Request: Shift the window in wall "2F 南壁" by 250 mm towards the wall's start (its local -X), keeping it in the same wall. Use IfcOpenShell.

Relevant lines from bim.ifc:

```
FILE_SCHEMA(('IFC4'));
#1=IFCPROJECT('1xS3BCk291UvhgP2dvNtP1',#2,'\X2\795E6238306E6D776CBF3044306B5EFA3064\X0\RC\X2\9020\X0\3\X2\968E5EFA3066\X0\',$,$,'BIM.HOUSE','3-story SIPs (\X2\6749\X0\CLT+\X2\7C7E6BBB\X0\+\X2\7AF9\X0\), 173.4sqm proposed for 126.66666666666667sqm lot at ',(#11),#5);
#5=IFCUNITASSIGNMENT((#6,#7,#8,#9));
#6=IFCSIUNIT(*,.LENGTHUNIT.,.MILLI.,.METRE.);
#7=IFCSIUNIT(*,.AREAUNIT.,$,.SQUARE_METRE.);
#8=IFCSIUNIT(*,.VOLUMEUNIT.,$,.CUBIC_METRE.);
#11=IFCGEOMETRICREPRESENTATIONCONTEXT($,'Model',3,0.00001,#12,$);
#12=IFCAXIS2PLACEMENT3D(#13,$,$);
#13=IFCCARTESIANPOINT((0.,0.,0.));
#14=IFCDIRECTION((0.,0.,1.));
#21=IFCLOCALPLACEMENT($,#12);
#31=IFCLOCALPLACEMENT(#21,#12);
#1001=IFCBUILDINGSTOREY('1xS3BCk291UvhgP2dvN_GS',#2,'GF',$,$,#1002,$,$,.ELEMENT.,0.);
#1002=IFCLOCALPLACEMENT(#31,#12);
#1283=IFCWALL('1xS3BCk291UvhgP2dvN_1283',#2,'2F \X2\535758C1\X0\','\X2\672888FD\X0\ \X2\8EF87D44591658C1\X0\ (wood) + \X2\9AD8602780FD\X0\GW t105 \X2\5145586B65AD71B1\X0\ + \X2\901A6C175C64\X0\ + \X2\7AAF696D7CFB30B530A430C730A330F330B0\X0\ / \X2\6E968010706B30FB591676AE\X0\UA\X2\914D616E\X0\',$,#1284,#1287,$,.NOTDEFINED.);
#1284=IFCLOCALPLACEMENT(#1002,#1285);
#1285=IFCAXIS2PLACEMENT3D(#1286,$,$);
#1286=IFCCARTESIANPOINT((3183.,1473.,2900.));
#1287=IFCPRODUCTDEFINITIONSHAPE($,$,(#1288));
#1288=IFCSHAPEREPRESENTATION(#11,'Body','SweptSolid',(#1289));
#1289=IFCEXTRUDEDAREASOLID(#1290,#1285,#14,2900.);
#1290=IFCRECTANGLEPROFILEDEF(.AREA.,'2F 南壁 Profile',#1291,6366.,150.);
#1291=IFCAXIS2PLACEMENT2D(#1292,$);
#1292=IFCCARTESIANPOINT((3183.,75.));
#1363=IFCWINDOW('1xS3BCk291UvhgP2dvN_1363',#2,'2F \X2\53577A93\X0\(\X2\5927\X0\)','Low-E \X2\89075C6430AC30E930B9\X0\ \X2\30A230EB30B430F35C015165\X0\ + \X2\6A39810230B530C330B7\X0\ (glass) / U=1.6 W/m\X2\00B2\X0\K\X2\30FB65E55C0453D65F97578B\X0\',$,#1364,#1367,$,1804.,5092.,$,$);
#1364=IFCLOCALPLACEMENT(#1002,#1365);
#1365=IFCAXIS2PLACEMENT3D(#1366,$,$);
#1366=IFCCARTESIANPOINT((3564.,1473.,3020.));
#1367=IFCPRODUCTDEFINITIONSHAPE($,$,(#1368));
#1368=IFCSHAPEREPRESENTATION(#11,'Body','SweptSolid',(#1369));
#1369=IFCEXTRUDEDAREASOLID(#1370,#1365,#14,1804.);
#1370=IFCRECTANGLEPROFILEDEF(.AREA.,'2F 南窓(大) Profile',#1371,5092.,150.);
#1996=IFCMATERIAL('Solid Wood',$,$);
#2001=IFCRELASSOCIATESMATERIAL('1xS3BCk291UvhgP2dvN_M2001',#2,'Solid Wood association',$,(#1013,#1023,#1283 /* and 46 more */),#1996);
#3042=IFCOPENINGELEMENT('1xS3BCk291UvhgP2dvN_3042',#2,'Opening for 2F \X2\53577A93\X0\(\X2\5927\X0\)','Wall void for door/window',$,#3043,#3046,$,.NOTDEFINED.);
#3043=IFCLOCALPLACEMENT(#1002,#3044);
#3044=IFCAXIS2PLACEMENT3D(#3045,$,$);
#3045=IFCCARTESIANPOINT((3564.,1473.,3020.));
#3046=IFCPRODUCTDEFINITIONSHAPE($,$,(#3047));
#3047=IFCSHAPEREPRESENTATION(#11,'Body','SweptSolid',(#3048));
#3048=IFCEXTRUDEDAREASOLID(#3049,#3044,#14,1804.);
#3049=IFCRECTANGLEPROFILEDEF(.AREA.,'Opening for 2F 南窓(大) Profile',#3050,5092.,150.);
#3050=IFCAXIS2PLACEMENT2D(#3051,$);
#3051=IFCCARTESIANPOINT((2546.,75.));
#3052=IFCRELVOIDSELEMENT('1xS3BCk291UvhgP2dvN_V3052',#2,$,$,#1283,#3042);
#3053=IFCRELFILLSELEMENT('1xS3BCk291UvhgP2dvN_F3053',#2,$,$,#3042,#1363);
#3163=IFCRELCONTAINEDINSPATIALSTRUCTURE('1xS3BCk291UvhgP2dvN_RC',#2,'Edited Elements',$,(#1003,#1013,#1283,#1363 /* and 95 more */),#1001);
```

```python
import ifcopenshell
import ifcopenshell.api.geometry
import ifcopenshell.util.placement
import ifcopenshell.util.unit

model = ifcopenshell.open("bim.ifc")
unit_scale = ifcopenshell.util.unit.calculate_unit_scale(model)

window = model.by_guid("1xS3BCk291UvhgP2dvN_1363")
opening = window.FillsVoids[0].RelatingOpeningElement
wall = opening.VoidsElements[0].RelatingBuildingElement

wall_matrix = ifcopenshell.util.placement.get_local_placement(wall.ObjectPlacement)
shift = wall_matrix[:3, 0] * -0.25 / unit_scale
before = ifcopenshell.util.placement.get_local_placement(window.ObjectPlacement)[:3, 3].copy()

# The window is not placed relative to its opening, so move both.
for product in (opening, window):
    matrix = ifcopenshell.util.placement.get_local_placement(product.ObjectPlacement)
    matrix[:3, 3] += shift
    ifcopenshell.api.geometry.edit_object_placement(model, product=product, matrix=matrix, is_si=False)

after = ifcopenshell.util.placement.get_local_placement(window.ObjectPlacement)[:3, 3]
print("window moved by", (after - before).round(3) + 0.0)

model.write("bim_rev.ifc")
```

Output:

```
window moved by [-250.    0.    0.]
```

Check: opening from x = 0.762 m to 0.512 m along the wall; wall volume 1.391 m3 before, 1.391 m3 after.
